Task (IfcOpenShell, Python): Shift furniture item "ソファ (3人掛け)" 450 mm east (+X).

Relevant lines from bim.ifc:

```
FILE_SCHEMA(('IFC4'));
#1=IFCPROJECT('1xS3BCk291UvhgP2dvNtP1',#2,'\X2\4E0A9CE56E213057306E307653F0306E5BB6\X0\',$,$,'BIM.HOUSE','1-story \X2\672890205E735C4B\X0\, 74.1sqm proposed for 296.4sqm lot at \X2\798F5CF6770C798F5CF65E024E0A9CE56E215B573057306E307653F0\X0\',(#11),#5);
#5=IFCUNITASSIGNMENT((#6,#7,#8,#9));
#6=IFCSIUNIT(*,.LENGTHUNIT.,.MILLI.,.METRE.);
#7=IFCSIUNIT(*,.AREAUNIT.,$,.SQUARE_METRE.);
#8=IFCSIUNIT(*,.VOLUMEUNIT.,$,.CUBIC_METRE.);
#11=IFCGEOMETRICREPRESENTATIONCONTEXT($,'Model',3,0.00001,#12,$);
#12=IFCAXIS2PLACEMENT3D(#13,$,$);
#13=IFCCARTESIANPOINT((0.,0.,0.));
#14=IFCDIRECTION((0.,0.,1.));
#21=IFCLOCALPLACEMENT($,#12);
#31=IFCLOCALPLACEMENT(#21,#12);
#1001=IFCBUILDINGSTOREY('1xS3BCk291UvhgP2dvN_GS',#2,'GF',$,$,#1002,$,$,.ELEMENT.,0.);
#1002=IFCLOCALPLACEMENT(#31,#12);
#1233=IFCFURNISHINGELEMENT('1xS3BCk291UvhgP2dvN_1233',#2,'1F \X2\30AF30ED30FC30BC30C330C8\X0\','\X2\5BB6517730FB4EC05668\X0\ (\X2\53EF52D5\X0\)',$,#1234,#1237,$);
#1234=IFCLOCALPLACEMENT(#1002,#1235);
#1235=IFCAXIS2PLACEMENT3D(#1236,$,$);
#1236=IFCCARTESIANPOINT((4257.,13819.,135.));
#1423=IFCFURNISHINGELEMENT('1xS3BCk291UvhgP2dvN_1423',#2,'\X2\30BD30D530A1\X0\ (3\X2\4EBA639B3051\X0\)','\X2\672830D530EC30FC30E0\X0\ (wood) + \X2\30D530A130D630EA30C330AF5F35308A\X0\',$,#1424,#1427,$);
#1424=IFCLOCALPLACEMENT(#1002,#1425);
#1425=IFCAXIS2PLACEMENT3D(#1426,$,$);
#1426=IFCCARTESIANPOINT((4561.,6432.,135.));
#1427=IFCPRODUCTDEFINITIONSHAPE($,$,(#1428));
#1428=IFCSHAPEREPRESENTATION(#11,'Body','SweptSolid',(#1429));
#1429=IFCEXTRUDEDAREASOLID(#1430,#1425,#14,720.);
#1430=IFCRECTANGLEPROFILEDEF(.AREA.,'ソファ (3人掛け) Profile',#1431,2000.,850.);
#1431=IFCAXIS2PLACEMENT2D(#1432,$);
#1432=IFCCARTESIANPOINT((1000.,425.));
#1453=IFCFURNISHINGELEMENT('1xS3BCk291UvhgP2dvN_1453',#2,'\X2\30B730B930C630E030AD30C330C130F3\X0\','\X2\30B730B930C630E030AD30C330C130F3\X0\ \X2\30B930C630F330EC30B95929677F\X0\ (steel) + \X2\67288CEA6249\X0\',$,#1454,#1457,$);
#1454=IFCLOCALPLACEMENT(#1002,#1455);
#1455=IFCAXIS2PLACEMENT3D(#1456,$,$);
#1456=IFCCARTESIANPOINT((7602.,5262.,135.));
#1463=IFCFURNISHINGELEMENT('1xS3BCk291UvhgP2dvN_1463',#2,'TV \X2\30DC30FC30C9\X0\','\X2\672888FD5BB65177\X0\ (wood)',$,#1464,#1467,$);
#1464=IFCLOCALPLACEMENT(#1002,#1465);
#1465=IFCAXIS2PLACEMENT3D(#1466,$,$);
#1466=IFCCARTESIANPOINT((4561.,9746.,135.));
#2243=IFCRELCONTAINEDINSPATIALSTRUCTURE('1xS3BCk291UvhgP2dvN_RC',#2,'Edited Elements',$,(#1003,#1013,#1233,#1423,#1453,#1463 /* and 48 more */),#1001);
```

```python
import ifcopenshell
import ifcopenshell.api.geometry
import ifcopenshell.util.placement
import ifcopenshell.util.unit

model = ifcopenshell.open("bim.ifc")
unit_scale = ifcopenshell.util.unit.calculate_unit_scale(model)

item = model.by_guid("1xS3BCk291UvhgP2dvN_1423")
matrix = ifcopenshell.util.placement.get_local_placement(item.ObjectPlacement)
matrix[0, 3] += 0.45 / unit_scale
ifcopenshell.api.geometry.edit_object_placement(model, product=item, matrix=matrix, is_si=False)

print(ifcopenshell.util.placement.get_local_placement(item.ObjectPlacement).round(3) + 0.0)

model.write("bim_updated.ifc")
```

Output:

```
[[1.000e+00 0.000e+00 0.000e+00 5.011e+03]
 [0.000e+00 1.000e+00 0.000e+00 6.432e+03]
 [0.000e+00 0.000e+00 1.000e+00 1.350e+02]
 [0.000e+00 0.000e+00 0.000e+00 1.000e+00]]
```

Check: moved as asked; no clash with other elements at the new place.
